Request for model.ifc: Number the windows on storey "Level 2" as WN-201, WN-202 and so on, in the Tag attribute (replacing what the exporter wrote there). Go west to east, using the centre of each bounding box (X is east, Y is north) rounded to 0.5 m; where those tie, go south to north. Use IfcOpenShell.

First a look at what the model holds.

```python
import ifcopenshell
import ifcopenshell.util.element
import ifcopenshell.util.placement

model = ifcopenshell.open("model.ifc")
print(model.schema)
storey = next(s for s in model.by_type("IfcBuildingStorey") if s.Name == "Level 2")
windows = [e for e in ifcopenshell.util.element.get_decomposition(storey) if e.is_a("IfcWindow")]
for e in sorted(windows, key=lambda e: e.id()):
    origin = ifcopenshell.util.placement.get_local_placement(e.ObjectPlacement)[:3, 3]
    print(e.id(), e.Tag, e.Name, origin.round(2) + 0.0, sep=" | ")
```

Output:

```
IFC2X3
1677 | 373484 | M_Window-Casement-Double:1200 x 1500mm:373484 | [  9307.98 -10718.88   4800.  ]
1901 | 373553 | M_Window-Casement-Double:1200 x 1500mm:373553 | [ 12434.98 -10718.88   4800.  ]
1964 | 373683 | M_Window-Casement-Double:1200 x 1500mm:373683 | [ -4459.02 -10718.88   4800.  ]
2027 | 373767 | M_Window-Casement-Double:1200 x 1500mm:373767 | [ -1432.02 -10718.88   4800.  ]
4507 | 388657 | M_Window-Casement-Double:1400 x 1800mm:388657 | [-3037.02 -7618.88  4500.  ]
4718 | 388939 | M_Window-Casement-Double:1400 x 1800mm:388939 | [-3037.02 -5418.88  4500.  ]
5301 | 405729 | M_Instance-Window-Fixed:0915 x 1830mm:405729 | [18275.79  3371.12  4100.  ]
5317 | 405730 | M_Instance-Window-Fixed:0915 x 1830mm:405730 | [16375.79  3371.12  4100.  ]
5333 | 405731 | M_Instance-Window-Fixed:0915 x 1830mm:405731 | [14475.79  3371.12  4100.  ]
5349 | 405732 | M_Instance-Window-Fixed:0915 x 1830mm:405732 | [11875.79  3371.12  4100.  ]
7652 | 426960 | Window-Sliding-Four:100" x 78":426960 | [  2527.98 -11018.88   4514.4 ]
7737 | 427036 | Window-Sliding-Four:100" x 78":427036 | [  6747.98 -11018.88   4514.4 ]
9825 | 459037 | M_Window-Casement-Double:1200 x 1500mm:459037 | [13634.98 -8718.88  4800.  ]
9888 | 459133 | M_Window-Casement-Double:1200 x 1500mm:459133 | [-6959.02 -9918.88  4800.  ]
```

```python
import ifcopenshell
import ifcopenshell.geom
import ifcopenshell.util.element
import ifcopenshell.util.shape

model = ifcopenshell.open("model.ifc")
settings = ifcopenshell.geom.settings()
settings.set("use-world-coords", True)


def centre(element):
    shape = ifcopenshell.geom.create_shape(settings, element)
    return ifcopenshell.util.shape.get_bbox_centroid(shape.geometry)


storey = next(s for s in model.by_type("IfcBuildingStorey") if s.Name == "Level 2")
windows = [e for e in ifcopenshell.util.element.get_decomposition(storey) if e.is_a("IfcWindow")]

# Insertion points can sit at a corner or the storey origin, so sort by the geometry (in metres).
centres = {e: centre(e) for e in windows}
windows.sort(key=lambda e: (round(centres[e][0] / 0.5), centres[e][1]))

for i, e in enumerate(windows, start=1):
    number = f"WN-2{i:02d}"
    e.Tag = number
    print(e.id(), number)

model.write("model-out.ifc")
```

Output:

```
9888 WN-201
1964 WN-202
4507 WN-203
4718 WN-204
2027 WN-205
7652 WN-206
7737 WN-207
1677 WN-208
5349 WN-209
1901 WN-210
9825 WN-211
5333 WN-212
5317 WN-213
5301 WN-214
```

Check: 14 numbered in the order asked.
